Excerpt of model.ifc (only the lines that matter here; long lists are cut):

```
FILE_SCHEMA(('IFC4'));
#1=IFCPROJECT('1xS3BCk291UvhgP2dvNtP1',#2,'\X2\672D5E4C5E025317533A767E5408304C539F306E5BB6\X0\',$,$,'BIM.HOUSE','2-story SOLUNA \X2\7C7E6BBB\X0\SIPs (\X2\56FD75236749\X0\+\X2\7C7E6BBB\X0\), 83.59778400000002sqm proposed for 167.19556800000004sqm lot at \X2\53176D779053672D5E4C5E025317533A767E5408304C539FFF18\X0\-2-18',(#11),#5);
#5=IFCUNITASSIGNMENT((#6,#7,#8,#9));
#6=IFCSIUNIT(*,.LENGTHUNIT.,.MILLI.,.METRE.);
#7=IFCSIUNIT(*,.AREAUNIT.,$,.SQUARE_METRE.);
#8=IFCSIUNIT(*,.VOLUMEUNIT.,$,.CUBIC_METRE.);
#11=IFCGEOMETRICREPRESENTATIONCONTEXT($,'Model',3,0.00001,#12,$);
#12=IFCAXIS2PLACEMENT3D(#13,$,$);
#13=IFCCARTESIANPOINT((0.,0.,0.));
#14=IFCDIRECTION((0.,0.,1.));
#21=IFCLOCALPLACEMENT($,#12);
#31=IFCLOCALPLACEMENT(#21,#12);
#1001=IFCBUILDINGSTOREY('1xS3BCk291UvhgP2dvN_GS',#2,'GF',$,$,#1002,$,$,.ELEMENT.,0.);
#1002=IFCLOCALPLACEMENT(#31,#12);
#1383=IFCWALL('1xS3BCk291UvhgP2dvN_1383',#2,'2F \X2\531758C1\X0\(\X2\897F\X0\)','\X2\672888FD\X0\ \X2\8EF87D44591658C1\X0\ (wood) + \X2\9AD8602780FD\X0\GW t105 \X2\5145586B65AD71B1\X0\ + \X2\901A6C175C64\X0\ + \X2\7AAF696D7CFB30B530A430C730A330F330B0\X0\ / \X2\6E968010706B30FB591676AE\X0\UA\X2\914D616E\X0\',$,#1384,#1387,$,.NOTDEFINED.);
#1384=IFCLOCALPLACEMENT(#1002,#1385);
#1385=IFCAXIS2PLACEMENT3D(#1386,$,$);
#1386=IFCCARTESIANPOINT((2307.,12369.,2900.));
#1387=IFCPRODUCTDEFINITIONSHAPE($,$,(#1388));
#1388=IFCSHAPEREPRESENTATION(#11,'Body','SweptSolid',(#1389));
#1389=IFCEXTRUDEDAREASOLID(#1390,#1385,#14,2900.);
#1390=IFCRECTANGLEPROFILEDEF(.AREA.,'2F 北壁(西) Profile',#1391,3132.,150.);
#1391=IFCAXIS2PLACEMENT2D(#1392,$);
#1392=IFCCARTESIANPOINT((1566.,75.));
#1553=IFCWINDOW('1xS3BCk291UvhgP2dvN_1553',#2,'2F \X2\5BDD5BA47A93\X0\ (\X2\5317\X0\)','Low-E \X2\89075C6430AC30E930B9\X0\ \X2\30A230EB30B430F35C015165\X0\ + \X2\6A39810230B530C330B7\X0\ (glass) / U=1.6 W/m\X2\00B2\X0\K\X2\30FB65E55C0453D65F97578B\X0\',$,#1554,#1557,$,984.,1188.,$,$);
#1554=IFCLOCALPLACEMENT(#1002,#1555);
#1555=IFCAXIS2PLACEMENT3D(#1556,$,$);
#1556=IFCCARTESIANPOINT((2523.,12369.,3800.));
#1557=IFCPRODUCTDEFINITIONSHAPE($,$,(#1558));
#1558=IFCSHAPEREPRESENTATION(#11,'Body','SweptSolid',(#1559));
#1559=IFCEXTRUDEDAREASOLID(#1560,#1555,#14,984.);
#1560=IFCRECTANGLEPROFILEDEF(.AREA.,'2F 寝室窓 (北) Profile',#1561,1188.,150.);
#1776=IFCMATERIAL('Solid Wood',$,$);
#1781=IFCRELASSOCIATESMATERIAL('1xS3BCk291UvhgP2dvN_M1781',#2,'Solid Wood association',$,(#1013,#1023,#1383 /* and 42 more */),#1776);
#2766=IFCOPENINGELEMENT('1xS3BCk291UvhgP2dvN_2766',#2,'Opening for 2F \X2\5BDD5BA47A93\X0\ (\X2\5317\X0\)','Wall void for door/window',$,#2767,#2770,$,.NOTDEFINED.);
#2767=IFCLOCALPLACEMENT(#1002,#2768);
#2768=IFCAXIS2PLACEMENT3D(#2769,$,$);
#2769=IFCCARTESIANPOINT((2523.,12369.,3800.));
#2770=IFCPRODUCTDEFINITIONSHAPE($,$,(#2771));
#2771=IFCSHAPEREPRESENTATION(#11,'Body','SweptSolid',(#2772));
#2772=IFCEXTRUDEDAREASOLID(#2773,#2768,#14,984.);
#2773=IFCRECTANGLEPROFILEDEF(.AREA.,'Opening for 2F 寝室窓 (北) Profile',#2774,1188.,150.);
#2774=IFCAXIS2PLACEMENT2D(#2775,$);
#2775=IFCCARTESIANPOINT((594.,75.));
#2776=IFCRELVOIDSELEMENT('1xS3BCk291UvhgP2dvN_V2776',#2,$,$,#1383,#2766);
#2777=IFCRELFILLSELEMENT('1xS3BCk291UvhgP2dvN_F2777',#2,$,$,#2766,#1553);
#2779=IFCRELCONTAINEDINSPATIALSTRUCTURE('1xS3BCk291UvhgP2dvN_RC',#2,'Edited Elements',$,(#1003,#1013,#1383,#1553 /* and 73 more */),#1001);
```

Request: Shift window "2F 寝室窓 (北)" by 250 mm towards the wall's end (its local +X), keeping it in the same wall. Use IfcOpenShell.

```python
import ifcopenshell
import ifcopenshell.api.geometry
import ifcopenshell.util.placement
import ifcopenshell.util.unit

model = ifcopenshell.open("model.ifc")
unit_scale = ifcopenshell.util.unit.calculate_unit_scale(model)

window = model.by_id(1553)
opening = window.FillsVoids[0].RelatingOpeningElement
wall = opening.VoidsElements[0].RelatingBuildingElement

wall_matrix = ifcopenshell.util.placement.get_local_placement(wall.ObjectPlacement)
shift = wall_matrix[:3, 0] * 0.25 / unit_scale
before = ifcopenshell.util.placement.get_local_placement(window.ObjectPlacement)[:3, 3].copy()

# The window is not placed relative to its opening, so move both.
for product in (opening, window):
    matrix = ifcopenshell.util.placement.get_local_placement(product.ObjectPlacement)
    matrix[:3, 3] += shift
    ifcopenshell.api.geometry.edit_object_placement(model, product=product, matrix=matrix, is_si=False)

after = ifcopenshell.util.placement.get_local_placement(window.ObjectPlacement)[:3, 3]
print("window moved by", (after - before).round(3) + 0.0)

model.write("model_v2.ifc")
```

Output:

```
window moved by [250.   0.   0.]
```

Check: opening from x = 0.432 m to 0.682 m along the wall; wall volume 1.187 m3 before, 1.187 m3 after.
